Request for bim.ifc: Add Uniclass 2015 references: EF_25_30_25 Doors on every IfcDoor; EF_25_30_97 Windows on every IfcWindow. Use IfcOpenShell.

First a look at what the model holds.

```python
import ifcopenshell

model = ifcopenshell.open("bim.ifc")
print(model.schema)
print("classifications:", [c.Name for c in model.by_type("IfcClassification")])
for ifc_class in ("IfcDoor", "IfcRoof", "IfcStair", "IfcWall", "IfcWindow"):
    print(ifc_class, len(model.by_type(ifc_class)))
```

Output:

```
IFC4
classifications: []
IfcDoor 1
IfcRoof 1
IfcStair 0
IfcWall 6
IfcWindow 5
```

```python
import ifcopenshell
import ifcopenshell.api.classification

model = ifcopenshell.open("bim.ifc")

system = ifcopenshell.api.classification.add_classification(model, classification="Uniclass 2015")

codes = {
    "IfcDoor": ("EF_25_30_25", "Doors"),
    "IfcWindow": ("EF_25_30_97", "Windows"),
}
for ifc_class, (code, name) in codes.items():
    products = model.by_type(ifc_class)
    ifcopenshell.api.classification.add_reference(
        model, products=products, classification=system, identification=code, name=name
    )
    print(code, len(products))

model.write("bim_rev.ifc")
```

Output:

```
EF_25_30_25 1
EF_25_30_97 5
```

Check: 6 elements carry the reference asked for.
